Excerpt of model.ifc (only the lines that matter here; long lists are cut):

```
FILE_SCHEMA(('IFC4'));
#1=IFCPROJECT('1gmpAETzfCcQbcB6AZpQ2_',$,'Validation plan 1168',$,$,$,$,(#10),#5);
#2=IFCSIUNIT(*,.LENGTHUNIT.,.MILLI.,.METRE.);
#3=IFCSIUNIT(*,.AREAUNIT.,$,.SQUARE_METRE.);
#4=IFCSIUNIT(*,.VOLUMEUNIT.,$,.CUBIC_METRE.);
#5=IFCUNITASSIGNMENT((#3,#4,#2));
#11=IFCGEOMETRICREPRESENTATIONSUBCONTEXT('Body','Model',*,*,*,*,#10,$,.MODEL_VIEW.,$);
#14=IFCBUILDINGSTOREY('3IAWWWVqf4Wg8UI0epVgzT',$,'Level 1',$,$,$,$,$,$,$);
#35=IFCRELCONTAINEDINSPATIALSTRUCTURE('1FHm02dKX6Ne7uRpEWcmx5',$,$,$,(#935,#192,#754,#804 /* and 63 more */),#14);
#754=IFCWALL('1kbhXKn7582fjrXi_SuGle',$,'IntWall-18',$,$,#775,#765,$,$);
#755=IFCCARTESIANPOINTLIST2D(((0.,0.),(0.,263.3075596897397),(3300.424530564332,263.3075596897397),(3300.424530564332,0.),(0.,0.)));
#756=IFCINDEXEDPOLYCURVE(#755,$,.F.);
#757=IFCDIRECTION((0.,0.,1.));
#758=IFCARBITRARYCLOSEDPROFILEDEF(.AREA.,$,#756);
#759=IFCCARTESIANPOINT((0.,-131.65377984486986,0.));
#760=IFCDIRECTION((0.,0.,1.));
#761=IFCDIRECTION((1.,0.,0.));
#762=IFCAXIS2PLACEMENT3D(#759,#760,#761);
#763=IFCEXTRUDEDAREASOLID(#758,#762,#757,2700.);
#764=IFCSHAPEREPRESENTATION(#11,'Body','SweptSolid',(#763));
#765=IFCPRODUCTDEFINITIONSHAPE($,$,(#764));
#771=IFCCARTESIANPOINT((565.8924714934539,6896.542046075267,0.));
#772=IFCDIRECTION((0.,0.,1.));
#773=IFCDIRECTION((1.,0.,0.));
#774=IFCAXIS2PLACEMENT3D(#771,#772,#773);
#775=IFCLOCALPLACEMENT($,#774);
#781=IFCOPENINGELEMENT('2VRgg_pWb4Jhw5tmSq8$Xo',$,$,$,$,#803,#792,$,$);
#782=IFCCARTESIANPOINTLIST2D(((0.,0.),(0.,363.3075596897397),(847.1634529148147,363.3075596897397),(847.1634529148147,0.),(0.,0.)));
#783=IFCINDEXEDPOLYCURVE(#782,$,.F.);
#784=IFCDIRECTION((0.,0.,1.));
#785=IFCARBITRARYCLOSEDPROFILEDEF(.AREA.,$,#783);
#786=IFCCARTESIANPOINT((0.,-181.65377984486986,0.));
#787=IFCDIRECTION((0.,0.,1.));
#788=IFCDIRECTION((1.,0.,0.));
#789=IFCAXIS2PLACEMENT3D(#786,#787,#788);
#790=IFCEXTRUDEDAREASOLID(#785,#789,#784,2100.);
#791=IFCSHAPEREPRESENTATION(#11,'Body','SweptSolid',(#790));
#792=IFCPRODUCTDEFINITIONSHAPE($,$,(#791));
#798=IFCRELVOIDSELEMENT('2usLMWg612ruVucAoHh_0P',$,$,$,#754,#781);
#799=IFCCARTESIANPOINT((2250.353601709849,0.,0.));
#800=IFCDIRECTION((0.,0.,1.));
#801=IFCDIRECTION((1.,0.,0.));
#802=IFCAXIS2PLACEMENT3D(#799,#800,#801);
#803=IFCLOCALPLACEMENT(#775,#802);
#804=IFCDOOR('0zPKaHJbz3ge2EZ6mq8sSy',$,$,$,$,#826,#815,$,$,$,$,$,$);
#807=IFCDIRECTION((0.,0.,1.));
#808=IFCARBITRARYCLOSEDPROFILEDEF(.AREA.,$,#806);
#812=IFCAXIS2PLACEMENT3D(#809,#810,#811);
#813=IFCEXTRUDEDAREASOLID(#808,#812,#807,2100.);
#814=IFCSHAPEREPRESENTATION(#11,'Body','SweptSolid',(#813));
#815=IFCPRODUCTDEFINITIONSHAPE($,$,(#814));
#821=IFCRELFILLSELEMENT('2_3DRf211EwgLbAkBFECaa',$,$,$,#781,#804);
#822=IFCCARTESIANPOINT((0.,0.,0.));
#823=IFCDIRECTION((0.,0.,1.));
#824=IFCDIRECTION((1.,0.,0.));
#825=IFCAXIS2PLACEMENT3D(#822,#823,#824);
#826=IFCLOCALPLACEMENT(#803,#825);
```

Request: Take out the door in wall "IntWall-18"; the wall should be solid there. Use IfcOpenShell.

```python
import ifcopenshell
import ifcopenshell.api.feature
import ifcopenshell.api.root
import ifcopenshell.geom
import ifcopenshell.util.shape

model = ifcopenshell.open("model.ifc")
settings = ifcopenshell.geom.settings()


def volume(element):
    """Net volume in cubic metres, openings subtracted."""
    shape = ifcopenshell.geom.create_shape(settings, element)
    return ifcopenshell.util.shape.get_volume(shape.geometry)


door = model.by_guid("0zPKaHJbz3ge2EZ6mq8sSy")
opening = door.FillsVoids[0].RelatingOpeningElement
wall = opening.VoidsElements[0].RelatingBuildingElement
before = volume(wall)

ifcopenshell.api.root.remove_product(model, product=door)
ifcopenshell.api.feature.remove_feature(model, feature=opening)

after = volume(wall)

print(f"wall volume {before:.3f} -> {after:.3f} m3")

model.write("model_v2.ifc")
```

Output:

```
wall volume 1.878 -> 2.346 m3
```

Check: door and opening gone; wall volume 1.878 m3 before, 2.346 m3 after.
